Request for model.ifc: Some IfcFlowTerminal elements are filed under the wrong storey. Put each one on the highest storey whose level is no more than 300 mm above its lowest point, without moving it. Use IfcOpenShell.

First a look at what the model holds.

```python
import ifcopenshell
import ifcopenshell.util.element
import ifcopenshell.util.placement

model = ifcopenshell.open("model.ifc")
print(model.schema)
for storey in model.by_type("IfcBuildingStorey"):
    level = ifcopenshell.util.placement.get_storey_elevation(storey)
    count = sum(e.is_a("IfcFlowTerminal") for e in ifcopenshell.util.element.get_contained(storey))
    print(storey.id(), storey.Name, round(level, 3), count, sep=" | ")
```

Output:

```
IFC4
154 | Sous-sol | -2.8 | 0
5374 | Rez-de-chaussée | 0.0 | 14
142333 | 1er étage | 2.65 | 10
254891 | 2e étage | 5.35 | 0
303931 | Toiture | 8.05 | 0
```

```python
import ifcopenshell
import ifcopenshell.api.spatial
import ifcopenshell.geom
import ifcopenshell.util.element
import ifcopenshell.util.placement
import ifcopenshell.util.shape
import ifcopenshell.util.unit

model = ifcopenshell.open("model.ifc")
unit_scale = ifcopenshell.util.unit.calculate_unit_scale(model)
settings = ifcopenshell.geom.settings()

levels = sorted(
    ((ifcopenshell.util.placement.get_storey_elevation(s) * unit_scale, s) for s in model.by_type("IfcBuildingStorey")),
    key=lambda pair: pair[0],
)

for e in model.by_type("IfcFlowTerminal"):
    current = e.ContainedInStructure[0].RelatingStructure if e.ContainedInStructure else None
    if current is None or not current.is_a("IfcBuildingStorey"):
        continue
    shape = ifcopenshell.geom.create_shape(settings, e)
    bottom = ifcopenshell.util.shape.get_shape_bottom_elevation(shape, shape.geometry)
    below = [s for level, s in levels if level <= bottom + 0.3]
    storey = below[-1] if below else levels[0][1]
    if storey != current:
        # assign_container keeps the world position.
        ifcopenshell.api.spatial.assign_container(model, products=[e], relating_structure=storey)
        print(e.id(), current.Name, "->", storey.Name)

model.write("model_v2.ifc")
```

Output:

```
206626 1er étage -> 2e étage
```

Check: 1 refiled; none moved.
